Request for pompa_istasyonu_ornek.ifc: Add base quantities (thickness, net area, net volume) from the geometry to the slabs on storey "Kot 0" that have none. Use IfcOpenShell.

First a look at what the model holds.

```python
import ifcopenshell
import ifcopenshell.util.element
import ifcopenshell.util.unit

model = ifcopenshell.open("pompa_istasyonu_ornek.ifc")
print(model.schema)
for unit_type in ("LENGTHUNIT", "AREAUNIT", "VOLUMEUNIT"):
    print(unit_type, ifcopenshell.util.unit.calculate_unit_scale(model, unit_type))
storey = next(s for s in model.by_type("IfcBuildingStorey") if s.Name == "Kot 0")
slabs = [e for e in ifcopenshell.util.element.get_decomposition(storey) if e.is_a("IfcSlab")]
for e in sorted(slabs, key=lambda e: e.id()):
    print(e.id(), e.is_a(), e.Name, list(ifcopenshell.util.element.get_psets(e, qtos_only=True)), sep=" | ")
```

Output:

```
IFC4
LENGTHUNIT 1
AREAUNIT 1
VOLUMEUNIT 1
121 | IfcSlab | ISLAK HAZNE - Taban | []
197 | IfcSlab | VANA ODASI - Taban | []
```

```python
import ifcopenshell
import ifcopenshell.api.pset
import ifcopenshell.geom
import ifcopenshell.util.element
import ifcopenshell.util.shape
import ifcopenshell.util.unit

model = ifcopenshell.open("pompa_istasyonu_ornek.ifc")
unit_scale = ifcopenshell.util.unit.calculate_unit_scale(model)
area_scale = ifcopenshell.util.unit.calculate_unit_scale(model, "AREAUNIT")
volume_scale = ifcopenshell.util.unit.calculate_unit_scale(model, "VOLUMEUNIT")
settings = ifcopenshell.geom.settings()

storey = next(s for s in model.by_type("IfcBuildingStorey") if s.Name == "Kot 0")
slabs = [e for e in ifcopenshell.util.element.get_decomposition(storey) if e.is_a("IfcSlab")]

for e in sorted(slabs, key=lambda e: e.id()):
    if ifcopenshell.util.element.get_psets(e, qtos_only=True, should_inherit=False):
        continue
    # Geometry comes back in metres, in the element's own axes.
    shape = ifcopenshell.geom.create_shape(settings, e)
    values = {
        "Width": ifcopenshell.util.shape.get_z(shape.geometry) / unit_scale,
        "NetArea": ifcopenshell.util.shape.get_footprint_area(shape.geometry) / area_scale,
        "NetVolume": ifcopenshell.util.shape.get_volume(shape.geometry) / volume_scale,
    }
    qto = ifcopenshell.api.pset.add_qto(model, product=e, name="Qto_SlabBaseQuantities")
    ifcopenshell.api.pset.edit_qto(model, qto=qto, properties=values)
    print(e.id(), {k: round(v, 3) for k, v in values.items()})

model.write("pompa_istasyonu_ornek_v2.ifc")
```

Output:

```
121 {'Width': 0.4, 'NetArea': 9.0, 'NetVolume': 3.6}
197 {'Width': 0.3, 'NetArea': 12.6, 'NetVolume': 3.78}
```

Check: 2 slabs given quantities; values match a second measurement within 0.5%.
